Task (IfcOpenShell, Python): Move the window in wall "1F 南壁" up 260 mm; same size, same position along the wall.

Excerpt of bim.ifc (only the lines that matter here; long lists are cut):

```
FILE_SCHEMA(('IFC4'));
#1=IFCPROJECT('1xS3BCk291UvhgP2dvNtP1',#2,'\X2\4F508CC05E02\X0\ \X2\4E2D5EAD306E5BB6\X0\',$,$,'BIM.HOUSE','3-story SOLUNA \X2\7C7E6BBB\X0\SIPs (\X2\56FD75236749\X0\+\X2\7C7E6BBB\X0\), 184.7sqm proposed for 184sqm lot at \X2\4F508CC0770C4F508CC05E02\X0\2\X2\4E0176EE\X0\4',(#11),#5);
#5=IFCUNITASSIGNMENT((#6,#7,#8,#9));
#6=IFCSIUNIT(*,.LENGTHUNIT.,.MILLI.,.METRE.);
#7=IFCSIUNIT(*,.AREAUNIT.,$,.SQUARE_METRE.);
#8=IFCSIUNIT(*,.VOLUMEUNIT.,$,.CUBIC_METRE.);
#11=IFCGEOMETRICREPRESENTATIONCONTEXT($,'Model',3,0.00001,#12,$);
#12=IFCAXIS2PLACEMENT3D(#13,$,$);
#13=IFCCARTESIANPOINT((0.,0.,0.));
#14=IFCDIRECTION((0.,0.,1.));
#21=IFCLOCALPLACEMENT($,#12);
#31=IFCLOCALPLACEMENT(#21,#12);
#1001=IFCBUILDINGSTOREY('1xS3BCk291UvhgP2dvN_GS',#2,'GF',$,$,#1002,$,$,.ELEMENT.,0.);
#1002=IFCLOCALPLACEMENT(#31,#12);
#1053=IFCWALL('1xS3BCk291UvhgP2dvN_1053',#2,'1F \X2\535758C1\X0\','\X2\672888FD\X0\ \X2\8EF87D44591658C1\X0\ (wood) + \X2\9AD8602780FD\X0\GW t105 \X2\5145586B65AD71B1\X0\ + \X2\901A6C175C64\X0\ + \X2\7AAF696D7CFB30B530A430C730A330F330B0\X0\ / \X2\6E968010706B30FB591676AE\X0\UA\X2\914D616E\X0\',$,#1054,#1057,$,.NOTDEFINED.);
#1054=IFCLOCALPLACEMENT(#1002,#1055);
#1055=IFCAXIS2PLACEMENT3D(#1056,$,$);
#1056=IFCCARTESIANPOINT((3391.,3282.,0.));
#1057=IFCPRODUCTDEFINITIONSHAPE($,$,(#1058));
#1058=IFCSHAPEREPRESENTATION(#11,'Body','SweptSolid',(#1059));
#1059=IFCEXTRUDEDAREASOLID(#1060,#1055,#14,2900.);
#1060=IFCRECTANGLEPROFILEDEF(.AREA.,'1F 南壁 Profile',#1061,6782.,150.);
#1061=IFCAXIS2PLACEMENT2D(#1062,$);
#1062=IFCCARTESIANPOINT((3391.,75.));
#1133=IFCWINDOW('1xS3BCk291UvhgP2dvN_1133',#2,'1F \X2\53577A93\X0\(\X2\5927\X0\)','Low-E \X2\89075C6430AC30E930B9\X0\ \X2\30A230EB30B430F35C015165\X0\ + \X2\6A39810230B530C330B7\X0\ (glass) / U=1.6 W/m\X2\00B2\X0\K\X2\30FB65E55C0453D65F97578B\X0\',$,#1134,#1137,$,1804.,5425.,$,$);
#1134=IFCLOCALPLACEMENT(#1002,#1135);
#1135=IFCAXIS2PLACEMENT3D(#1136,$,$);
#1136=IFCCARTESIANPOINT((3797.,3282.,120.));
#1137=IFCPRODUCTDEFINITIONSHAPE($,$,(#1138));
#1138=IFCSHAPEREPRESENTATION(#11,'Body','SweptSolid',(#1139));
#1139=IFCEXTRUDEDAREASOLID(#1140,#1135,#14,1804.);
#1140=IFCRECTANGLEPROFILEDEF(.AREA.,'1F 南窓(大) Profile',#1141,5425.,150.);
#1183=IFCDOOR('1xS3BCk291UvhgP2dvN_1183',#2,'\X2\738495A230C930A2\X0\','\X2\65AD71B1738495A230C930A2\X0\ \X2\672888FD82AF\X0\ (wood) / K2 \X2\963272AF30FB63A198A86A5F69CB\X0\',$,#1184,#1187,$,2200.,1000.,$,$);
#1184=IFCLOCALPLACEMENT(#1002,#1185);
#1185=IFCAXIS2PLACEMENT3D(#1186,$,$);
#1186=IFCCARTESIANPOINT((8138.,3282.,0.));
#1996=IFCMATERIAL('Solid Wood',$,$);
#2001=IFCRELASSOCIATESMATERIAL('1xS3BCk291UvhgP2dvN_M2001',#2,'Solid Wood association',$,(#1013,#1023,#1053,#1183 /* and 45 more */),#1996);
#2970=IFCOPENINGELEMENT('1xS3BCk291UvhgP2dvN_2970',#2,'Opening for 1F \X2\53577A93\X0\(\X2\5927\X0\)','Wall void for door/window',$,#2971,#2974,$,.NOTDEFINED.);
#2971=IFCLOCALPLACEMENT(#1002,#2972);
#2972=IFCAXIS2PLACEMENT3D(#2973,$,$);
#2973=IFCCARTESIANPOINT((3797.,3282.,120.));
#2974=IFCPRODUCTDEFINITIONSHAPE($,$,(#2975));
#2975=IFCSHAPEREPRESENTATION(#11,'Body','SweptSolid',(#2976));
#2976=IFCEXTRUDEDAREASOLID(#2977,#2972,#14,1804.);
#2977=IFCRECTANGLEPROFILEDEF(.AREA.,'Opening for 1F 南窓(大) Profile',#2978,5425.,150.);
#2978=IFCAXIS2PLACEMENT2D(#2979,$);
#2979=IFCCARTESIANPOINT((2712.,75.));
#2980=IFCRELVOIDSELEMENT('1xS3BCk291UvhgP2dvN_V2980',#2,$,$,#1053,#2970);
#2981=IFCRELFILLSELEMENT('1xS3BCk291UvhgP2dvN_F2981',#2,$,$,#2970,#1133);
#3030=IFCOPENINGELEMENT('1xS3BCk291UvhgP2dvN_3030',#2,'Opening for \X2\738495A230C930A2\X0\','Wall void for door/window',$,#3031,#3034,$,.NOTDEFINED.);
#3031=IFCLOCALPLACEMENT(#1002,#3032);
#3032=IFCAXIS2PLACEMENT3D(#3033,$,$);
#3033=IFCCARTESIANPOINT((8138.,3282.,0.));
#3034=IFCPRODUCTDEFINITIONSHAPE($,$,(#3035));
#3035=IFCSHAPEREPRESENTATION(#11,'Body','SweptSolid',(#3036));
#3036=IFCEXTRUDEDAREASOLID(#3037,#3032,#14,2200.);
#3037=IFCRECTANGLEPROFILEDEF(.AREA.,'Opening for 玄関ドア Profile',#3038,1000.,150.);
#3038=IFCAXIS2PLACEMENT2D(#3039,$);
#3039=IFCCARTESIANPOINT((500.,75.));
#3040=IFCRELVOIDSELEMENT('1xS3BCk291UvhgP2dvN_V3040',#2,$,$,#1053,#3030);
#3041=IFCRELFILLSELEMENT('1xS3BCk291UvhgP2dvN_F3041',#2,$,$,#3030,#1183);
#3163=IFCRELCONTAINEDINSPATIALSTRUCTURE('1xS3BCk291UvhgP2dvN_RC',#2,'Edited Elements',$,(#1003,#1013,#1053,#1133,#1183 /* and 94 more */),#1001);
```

```python
import numpy as np
import ifcopenshell
import ifcopenshell.api.geometry
import ifcopenshell.util.placement
import ifcopenshell.util.unit

model = ifcopenshell.open("bim.ifc")
unit_scale = ifcopenshell.util.unit.calculate_unit_scale(model)

window = model.by_guid("1xS3BCk291UvhgP2dvN_1133")
opening = window.FillsVoids[0].RelatingOpeningElement
dz = 0.26 / unit_scale

shift = np.array([0.0, 0.0, dz])
# The window is not placed relative to its opening, so move both.
for product in (opening, window):
    matrix = ifcopenshell.util.placement.get_local_placement(product.ObjectPlacement)
    matrix[:3, 3] += shift
    ifcopenshell.api.geometry.edit_object_placement(model, product=product, matrix=matrix, is_si=False)

print(f"moved by {dz * unit_scale:+.3f} m")

model.write("bim_updated.ifc")
```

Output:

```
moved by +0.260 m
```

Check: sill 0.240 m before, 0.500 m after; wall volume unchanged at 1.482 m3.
